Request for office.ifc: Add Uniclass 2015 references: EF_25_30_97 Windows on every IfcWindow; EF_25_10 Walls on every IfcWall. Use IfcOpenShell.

First a look at what the model holds.

```python
import ifcopenshell

model = ifcopenshell.open("office.ifc")
print(model.schema)
print("classifications:", [c.Name for c in model.by_type("IfcClassification")])
for ifc_class in ("IfcDoor", "IfcRoof", "IfcStair", "IfcWall", "IfcWindow"):
    print(ifc_class, len(model.by_type(ifc_class)))
```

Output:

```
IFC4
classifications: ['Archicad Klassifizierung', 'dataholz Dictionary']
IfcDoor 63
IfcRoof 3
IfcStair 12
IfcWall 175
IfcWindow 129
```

```python
import ifcopenshell
import ifcopenshell.api.classification

model = ifcopenshell.open("office.ifc")

system = ifcopenshell.api.classification.add_classification(model, classification="Uniclass 2015")

codes = {
    "IfcWindow": ("EF_25_30_97", "Windows"),
    "IfcWall": ("EF_25_10", "Walls"),
}
for ifc_class, (code, name) in codes.items():
    products = model.by_type(ifc_class)
    ifcopenshell.api.classification.add_reference(
        model, products=products, classification=system, identification=code, name=name
    )
    print(code, len(products))

model.write("office_rev.ifc")
```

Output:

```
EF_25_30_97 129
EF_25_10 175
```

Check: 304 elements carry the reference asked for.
